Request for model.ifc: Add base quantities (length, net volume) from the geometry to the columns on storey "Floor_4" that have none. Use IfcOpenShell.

First a look at what the model holds.

```python
import ifcopenshell
import ifcopenshell.util.element
import ifcopenshell.util.unit

model = ifcopenshell.open("model.ifc")
print(model.schema)
for unit_type in ("LENGTHUNIT", "AREAUNIT", "VOLUMEUNIT"):
    print(unit_type, ifcopenshell.util.unit.calculate_unit_scale(model, unit_type))
storey = next(s for s in model.by_type("IfcBuildingStorey") if s.Name == "Floor_4")
columns = [e for e in ifcopenshell.util.element.get_decomposition(storey) if e.is_a("IfcColumn")]
for e in sorted(columns, key=lambda e: e.id()):
    print(e.id(), e.is_a(), e.Name, list(ifcopenshell.util.element.get_psets(e, qtos_only=True)), sep=" | ")
```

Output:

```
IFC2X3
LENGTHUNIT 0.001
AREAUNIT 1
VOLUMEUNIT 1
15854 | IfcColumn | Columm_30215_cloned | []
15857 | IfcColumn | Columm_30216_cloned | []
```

```python
import ifcopenshell
import ifcopenshell.api.pset
import ifcopenshell.geom
import ifcopenshell.util.element
import ifcopenshell.util.shape
import ifcopenshell.util.unit

model = ifcopenshell.open("model.ifc")
unit_scale = ifcopenshell.util.unit.calculate_unit_scale(model)
volume_scale = ifcopenshell.util.unit.calculate_unit_scale(model, "VOLUMEUNIT")
settings = ifcopenshell.geom.settings()

storey = next(s for s in model.by_type("IfcBuildingStorey") if s.Name == "Floor_4")
columns = [e for e in ifcopenshell.util.element.get_decomposition(storey) if e.is_a("IfcColumn")]

for e in sorted(columns, key=lambda e: e.id()):
    if ifcopenshell.util.element.get_psets(e, qtos_only=True, should_inherit=False):
        continue
    # Geometry comes back in metres, in the element's own axes.
    shape = ifcopenshell.geom.create_shape(settings, e)
    values = {
        "Length": ifcopenshell.util.shape.get_z(shape.geometry) / unit_scale,
        "NetVolume": ifcopenshell.util.shape.get_volume(shape.geometry) / volume_scale,
    }
    qto = ifcopenshell.api.pset.add_qto(model, product=e, name="BaseQuantities")
    ifcopenshell.api.pset.edit_qto(model, qto=qto, properties=values)
    print(e.id(), {k: round(v, 3) for k, v in values.items()})

model.write("model-out.ifc")
```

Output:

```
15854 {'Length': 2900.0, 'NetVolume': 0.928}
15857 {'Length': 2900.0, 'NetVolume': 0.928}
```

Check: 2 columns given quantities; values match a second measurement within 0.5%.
